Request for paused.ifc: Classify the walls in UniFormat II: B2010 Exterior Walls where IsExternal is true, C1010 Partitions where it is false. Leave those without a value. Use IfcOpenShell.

First a look at what the model holds.

```python
import ifcopenshell
import ifcopenshell.util.element

model = ifcopenshell.open("paused.ifc")
print(model.schema)
print("classifications:", [c.Name for c in model.by_type("IfcClassification")])
values = [ifcopenshell.util.element.get_pset(e, "Pset_WallCommon", "IsExternal") for e in model.by_type("IfcWall")]
for value in (True, False, None):
    print("IsExternal", value, values.count(value))
```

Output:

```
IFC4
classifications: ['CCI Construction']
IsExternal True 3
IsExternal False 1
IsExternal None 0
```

```python
import ifcopenshell
import ifcopenshell.api.classification
import ifcopenshell.util.element

model = ifcopenshell.open("paused.ifc")

system = ifcopenshell.api.classification.add_classification(model, classification="UniFormat II")

walls = model.by_type("IfcWall")
external = {e: ifcopenshell.util.element.get_pset(e, "Pset_WallCommon", "IsExternal") for e in walls}
for flag, code, name in ((True, "B2010", "Exterior Walls"), (False, "C1010", "Partitions")):
    products = [e for e in walls if external[e] is flag]
    ifcopenshell.api.classification.add_reference(
        model, products=products, classification=system, identification=code, name=name
    )
    print(code, len(products))

model.write("paused-out.ifc")
```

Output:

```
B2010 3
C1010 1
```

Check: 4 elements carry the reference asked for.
